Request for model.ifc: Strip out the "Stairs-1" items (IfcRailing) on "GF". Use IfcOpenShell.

First a look at what the model holds.

```python
import ifcopenshell
import ifcopenshell.util.element

model = ifcopenshell.open("model.ifc")
print(model.schema)
storey = next(s for s in model.by_type("IfcBuildingStorey") if s.Name == "GF")
railings = [e for e in ifcopenshell.util.element.get_decomposition(storey) if e.is_a("IfcRailing")]
seen = {}
for e in railings:
    element_type = ifcopenshell.util.element.get_type(e)
    name = element_type.Name if element_type not in (None, e) else None
    seen[name] = seen.get(name, 0) + 1
for name, count in sorted(seen.items(), key=str):
    print(count, "x", name)
```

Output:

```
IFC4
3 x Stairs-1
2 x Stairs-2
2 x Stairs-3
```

```python
import ifcopenshell
import ifcopenshell.api.root
import ifcopenshell.util.element

model = ifcopenshell.open("model.ifc")

storey = next(s for s in model.by_type("IfcBuildingStorey") if s.Name == "GF")
railings = [e for e in ifcopenshell.util.element.get_decomposition(storey) if e.is_a("IfcRailing")]
targets = [e for e in railings if (t := ifcopenshell.util.element.get_type(e)) not in (None, e) and t.Name == "Stairs-1"]

for e in targets:
    ifcopenshell.api.root.remove_product(model, product=e)
print(len(targets), "removed")

model.write("model_rev.ifc")
```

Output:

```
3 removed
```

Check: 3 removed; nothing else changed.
